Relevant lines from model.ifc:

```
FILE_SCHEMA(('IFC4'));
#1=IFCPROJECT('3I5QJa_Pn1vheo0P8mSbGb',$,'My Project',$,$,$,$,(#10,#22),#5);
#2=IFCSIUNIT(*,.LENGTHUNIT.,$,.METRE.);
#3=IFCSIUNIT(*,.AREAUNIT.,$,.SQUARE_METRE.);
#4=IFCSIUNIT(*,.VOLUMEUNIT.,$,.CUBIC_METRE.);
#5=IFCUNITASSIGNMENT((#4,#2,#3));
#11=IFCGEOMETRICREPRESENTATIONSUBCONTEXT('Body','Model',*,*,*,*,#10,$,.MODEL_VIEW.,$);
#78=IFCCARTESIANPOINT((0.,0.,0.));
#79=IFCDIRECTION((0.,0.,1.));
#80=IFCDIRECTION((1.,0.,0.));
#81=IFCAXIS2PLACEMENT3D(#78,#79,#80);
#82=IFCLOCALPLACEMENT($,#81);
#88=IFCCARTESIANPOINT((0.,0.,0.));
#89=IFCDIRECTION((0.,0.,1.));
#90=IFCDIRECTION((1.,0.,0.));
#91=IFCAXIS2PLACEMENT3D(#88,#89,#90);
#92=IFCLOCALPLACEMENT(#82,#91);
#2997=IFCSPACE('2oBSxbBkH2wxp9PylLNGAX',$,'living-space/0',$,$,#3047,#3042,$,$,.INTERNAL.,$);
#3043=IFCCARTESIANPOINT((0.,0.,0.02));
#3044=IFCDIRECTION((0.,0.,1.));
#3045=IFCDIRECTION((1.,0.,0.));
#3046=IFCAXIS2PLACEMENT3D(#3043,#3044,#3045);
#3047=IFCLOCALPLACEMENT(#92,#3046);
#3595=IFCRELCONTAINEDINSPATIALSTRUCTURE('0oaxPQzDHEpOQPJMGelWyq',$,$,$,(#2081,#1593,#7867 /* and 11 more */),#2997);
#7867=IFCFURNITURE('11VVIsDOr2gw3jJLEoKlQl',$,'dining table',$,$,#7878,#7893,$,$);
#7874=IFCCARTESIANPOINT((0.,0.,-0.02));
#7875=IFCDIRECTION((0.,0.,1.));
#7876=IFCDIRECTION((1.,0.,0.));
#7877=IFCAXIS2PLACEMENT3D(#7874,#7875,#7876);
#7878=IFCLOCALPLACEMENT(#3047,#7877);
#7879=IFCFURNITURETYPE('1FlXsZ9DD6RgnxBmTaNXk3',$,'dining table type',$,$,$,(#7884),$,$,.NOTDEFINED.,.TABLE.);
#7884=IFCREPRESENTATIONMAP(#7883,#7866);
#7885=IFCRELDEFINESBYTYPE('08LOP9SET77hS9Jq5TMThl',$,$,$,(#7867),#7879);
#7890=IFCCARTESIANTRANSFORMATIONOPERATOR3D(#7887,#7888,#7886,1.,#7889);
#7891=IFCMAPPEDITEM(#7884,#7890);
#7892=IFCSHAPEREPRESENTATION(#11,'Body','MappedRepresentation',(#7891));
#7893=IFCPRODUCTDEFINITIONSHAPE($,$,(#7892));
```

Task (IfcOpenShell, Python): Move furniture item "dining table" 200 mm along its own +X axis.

```python
import ifcopenshell
import ifcopenshell.api.geometry
import ifcopenshell.util.placement
import ifcopenshell.util.unit

model = ifcopenshell.open("model.ifc")
unit_scale = ifcopenshell.util.unit.calculate_unit_scale(model)

item = model.by_id(7867)
matrix = ifcopenshell.util.placement.get_local_placement(item.ObjectPlacement)
matrix[:3, 3] += matrix[:3, 0] * 0.2 / unit_scale
ifcopenshell.api.geometry.edit_object_placement(model, product=item, matrix=matrix, is_si=False)

print(ifcopenshell.util.placement.get_local_placement(item.ObjectPlacement).round(3) + 0.0)

model.write("model_v2.ifc")
```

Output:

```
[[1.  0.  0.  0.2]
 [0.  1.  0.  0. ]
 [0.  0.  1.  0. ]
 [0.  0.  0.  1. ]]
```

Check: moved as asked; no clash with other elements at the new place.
